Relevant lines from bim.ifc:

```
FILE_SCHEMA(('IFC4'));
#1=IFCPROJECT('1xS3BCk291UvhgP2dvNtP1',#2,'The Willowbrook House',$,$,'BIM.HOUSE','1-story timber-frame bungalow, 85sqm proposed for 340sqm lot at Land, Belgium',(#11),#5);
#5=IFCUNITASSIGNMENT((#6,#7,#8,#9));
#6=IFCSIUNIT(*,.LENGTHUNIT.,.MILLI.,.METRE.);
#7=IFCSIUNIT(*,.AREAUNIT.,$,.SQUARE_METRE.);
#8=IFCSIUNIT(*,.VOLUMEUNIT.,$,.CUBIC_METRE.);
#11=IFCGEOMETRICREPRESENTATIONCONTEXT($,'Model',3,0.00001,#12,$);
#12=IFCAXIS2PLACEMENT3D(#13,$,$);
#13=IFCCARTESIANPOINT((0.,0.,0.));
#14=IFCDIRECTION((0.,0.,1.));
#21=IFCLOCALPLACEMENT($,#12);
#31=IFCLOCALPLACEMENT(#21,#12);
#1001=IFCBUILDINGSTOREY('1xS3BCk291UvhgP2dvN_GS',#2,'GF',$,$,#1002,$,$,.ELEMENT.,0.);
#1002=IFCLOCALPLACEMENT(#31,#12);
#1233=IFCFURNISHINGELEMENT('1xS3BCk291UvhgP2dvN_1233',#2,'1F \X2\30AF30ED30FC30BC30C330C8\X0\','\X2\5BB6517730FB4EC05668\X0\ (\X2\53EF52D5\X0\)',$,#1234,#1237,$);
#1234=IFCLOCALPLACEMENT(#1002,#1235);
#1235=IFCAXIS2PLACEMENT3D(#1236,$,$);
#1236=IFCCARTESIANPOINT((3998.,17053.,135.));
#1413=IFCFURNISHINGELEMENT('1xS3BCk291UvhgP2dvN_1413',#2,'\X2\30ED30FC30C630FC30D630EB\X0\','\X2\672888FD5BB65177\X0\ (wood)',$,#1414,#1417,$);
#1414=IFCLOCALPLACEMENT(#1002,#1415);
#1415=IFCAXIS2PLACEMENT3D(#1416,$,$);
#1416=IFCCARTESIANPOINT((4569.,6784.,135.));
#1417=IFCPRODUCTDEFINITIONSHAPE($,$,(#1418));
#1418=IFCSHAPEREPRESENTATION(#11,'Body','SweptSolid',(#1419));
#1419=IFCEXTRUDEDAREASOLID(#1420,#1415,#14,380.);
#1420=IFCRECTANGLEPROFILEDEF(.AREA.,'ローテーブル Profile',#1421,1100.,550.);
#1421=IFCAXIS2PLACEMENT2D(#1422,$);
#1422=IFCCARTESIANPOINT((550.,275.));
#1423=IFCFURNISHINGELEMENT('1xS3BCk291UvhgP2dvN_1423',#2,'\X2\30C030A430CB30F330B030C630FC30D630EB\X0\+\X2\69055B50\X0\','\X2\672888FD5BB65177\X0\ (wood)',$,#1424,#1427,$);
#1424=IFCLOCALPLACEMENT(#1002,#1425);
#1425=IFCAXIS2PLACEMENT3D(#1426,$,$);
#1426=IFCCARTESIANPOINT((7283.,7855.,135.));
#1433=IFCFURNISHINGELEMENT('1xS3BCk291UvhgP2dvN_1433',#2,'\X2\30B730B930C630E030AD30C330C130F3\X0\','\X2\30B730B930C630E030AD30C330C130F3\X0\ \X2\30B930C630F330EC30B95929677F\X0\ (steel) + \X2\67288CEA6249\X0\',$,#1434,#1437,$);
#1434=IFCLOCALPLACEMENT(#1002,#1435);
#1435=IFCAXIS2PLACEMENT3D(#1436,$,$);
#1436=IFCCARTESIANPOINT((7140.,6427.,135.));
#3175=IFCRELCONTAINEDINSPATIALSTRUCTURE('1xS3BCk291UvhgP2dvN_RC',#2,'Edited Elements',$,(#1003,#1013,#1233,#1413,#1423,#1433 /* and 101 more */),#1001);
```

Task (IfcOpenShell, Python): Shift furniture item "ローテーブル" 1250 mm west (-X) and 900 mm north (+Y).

```python
import ifcopenshell
import ifcopenshell.api.geometry
import ifcopenshell.util.placement
import ifcopenshell.util.unit

model = ifcopenshell.open("bim.ifc")
unit_scale = ifcopenshell.util.unit.calculate_unit_scale(model)

item = model.by_guid("1xS3BCk291UvhgP2dvN_1413")
matrix = ifcopenshell.util.placement.get_local_placement(item.ObjectPlacement)
matrix[0, 3] -= 1.25 / unit_scale
matrix[1, 3] += 0.9 / unit_scale
ifcopenshell.api.geometry.edit_object_placement(model, product=item, matrix=matrix, is_si=False)

print(ifcopenshell.util.placement.get_local_placement(item.ObjectPlacement).round(3) + 0.0)

model.write("bim_updated.ifc")
```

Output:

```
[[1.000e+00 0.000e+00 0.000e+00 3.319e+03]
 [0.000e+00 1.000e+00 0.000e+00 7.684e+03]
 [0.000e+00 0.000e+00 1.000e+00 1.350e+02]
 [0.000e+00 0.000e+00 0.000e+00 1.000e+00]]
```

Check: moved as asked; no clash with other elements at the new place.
